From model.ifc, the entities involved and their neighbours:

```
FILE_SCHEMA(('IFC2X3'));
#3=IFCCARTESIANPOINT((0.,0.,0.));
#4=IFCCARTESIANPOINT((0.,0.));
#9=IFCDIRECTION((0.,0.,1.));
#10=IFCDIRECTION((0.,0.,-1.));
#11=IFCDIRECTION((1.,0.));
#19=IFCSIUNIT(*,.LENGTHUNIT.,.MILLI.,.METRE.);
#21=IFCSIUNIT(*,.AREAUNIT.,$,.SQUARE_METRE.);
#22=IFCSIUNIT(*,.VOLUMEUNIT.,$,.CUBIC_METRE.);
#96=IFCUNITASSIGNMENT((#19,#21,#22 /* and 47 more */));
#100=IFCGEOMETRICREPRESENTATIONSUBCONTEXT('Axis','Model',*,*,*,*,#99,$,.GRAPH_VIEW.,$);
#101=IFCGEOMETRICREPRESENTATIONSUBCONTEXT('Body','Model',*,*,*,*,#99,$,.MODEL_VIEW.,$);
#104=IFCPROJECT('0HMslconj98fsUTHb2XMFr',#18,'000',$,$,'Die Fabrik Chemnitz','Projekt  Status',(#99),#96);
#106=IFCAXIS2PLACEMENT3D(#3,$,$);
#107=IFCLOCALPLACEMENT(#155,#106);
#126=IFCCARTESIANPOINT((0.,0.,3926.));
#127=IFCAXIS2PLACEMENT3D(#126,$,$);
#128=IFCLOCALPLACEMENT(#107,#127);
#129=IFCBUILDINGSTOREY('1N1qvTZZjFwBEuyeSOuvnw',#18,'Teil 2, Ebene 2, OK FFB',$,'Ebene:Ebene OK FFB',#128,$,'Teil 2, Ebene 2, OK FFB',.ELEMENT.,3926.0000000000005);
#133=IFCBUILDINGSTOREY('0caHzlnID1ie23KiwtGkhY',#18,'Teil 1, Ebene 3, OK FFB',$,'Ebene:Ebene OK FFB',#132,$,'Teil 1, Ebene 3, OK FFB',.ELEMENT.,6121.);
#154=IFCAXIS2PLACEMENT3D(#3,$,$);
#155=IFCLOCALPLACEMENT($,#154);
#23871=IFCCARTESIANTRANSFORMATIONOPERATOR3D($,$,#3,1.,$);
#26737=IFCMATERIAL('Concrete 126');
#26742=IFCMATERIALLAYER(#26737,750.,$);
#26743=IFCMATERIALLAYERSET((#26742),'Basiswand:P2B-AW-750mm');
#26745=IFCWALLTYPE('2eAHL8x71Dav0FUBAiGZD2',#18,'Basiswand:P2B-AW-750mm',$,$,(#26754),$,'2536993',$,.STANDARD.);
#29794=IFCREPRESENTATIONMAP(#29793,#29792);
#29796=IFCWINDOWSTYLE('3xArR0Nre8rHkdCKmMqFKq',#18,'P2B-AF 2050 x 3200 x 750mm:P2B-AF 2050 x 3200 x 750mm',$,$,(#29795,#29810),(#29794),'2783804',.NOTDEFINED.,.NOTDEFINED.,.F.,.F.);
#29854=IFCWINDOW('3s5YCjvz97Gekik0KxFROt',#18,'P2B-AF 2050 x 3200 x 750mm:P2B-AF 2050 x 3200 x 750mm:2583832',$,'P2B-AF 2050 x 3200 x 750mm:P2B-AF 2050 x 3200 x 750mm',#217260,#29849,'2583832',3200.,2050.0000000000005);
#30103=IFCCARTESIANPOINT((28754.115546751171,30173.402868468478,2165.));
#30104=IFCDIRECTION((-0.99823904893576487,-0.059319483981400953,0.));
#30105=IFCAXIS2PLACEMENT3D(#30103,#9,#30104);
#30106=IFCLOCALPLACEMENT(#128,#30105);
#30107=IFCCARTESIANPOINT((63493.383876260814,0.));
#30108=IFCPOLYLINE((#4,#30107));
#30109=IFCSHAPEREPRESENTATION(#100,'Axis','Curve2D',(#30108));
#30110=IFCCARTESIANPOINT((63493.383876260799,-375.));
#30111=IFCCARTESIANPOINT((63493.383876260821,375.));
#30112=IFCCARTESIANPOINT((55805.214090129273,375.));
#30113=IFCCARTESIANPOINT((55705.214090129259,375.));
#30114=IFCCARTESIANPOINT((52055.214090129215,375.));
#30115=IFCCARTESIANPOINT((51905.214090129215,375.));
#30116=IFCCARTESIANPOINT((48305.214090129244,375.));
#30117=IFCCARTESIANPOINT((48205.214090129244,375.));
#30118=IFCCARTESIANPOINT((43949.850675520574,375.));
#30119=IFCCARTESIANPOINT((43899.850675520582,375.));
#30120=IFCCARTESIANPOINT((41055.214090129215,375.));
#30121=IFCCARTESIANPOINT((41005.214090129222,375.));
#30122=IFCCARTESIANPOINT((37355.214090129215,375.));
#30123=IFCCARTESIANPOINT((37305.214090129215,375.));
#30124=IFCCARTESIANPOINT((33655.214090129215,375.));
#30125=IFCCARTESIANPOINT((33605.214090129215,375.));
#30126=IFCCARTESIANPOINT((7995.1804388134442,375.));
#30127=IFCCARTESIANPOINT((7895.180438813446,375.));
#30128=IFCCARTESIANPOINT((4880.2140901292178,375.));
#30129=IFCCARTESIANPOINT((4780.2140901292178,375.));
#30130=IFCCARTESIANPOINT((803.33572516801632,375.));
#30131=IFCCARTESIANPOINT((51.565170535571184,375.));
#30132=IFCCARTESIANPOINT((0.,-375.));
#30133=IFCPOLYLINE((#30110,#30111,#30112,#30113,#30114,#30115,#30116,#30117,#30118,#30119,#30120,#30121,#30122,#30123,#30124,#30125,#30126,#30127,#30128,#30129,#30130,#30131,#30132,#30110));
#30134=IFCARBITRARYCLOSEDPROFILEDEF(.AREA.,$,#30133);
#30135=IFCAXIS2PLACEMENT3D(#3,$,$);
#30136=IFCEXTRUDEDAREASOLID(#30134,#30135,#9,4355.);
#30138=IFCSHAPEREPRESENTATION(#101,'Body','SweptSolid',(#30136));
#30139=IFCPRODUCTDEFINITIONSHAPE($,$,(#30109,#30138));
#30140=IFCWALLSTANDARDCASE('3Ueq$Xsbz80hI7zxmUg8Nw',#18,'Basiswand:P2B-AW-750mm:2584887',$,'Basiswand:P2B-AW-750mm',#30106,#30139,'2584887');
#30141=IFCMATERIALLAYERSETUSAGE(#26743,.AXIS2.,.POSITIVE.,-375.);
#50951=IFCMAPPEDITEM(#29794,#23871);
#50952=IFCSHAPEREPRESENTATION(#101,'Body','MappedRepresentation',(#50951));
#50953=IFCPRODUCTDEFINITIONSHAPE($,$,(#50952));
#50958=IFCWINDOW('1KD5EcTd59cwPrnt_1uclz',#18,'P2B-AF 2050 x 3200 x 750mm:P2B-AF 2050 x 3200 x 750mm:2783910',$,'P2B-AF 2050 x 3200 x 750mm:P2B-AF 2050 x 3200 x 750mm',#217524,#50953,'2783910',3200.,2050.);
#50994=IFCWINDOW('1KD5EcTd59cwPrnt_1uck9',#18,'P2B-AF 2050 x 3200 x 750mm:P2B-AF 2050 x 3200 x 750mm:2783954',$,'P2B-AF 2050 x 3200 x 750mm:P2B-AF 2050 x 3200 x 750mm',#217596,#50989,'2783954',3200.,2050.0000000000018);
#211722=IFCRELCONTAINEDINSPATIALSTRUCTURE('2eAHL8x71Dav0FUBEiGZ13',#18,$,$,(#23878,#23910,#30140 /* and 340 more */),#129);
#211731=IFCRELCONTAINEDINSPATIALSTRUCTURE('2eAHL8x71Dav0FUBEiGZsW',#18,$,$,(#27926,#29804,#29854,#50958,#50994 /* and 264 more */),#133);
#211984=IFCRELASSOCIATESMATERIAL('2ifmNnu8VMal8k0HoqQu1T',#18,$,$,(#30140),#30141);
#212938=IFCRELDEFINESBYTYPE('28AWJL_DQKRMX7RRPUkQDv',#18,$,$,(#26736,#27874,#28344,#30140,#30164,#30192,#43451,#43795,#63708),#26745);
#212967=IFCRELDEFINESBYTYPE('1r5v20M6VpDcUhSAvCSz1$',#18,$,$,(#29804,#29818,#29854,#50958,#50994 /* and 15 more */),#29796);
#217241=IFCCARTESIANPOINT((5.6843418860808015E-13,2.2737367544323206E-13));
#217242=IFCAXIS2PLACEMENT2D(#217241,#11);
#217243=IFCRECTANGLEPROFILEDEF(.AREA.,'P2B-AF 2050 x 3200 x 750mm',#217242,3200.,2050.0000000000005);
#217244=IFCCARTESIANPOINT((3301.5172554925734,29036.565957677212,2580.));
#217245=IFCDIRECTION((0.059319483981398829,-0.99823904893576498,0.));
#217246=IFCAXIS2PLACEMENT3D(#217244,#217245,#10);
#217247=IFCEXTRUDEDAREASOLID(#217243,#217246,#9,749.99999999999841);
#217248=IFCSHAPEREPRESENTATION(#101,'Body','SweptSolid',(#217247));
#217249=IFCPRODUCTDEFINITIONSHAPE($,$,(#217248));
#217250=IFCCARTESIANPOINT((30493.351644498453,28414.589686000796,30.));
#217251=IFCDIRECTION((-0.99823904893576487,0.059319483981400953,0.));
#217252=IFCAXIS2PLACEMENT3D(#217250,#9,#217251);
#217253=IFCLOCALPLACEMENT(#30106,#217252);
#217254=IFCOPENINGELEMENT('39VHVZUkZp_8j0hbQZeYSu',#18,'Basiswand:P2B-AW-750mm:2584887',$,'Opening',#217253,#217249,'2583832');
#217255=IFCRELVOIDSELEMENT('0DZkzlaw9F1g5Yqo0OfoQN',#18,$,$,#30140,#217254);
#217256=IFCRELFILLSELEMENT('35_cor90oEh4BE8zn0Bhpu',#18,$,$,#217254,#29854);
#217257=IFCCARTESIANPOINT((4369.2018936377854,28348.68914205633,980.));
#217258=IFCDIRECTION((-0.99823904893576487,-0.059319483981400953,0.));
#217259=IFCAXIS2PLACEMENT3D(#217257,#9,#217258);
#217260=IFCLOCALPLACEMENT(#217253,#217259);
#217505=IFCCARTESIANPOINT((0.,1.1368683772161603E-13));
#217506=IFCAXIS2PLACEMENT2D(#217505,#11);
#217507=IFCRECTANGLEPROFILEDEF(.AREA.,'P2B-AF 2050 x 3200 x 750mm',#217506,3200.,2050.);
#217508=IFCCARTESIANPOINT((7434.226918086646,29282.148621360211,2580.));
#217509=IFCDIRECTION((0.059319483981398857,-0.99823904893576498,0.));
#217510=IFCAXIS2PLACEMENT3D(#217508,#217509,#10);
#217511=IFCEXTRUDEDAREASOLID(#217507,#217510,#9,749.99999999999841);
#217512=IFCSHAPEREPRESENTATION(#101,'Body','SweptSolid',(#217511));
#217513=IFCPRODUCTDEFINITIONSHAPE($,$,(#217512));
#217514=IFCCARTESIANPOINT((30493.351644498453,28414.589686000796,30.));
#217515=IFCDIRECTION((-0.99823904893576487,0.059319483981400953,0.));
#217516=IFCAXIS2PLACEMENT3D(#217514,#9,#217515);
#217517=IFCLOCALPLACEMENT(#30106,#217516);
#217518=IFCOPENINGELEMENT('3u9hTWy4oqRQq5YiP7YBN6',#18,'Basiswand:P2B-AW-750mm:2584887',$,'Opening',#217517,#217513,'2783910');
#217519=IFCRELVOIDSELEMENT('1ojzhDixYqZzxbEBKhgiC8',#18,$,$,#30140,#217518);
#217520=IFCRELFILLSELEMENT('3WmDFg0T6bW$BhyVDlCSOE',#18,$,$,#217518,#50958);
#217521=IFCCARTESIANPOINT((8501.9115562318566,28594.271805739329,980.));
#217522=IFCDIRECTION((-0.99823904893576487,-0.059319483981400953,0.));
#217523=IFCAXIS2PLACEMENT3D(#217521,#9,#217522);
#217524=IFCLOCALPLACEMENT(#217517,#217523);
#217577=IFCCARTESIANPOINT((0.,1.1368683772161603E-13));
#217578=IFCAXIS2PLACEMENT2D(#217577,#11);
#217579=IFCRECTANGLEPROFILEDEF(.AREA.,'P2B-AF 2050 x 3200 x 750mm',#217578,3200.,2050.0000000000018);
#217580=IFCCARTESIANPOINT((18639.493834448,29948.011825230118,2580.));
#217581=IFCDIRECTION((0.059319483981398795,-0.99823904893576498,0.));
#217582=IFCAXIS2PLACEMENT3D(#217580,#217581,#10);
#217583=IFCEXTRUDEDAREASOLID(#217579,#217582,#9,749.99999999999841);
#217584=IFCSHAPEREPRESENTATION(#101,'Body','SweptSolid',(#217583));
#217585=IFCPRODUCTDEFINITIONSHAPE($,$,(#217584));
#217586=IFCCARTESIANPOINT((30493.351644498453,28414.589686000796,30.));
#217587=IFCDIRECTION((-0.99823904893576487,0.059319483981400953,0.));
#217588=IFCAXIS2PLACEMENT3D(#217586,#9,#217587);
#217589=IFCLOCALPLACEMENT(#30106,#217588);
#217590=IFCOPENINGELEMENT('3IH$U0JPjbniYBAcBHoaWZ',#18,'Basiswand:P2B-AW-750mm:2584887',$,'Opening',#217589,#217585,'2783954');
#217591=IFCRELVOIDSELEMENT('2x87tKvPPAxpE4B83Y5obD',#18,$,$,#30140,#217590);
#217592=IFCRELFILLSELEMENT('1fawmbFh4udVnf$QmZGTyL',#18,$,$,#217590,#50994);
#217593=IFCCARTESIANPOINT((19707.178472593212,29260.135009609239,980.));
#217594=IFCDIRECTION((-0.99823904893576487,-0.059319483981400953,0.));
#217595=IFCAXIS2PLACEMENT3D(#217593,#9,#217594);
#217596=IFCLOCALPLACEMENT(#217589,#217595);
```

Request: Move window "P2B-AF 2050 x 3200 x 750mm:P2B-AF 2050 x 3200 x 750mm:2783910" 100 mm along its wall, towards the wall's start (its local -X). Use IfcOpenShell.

```python
import ifcopenshell
import ifcopenshell.api.geometry
import ifcopenshell.util.placement
import ifcopenshell.util.unit

model = ifcopenshell.open("model.ifc")
unit_scale = ifcopenshell.util.unit.calculate_unit_scale(model)

window = model.by_guid("1KD5EcTd59cwPrnt_1uclz")
opening = window.FillsVoids[0].RelatingOpeningElement
wall = opening.VoidsElements[0].RelatingBuildingElement

wall_matrix = ifcopenshell.util.placement.get_local_placement(wall.ObjectPlacement)
shift = wall_matrix[:3, 0] * -0.1 / unit_scale
before = ifcopenshell.util.placement.get_local_placement(window.ObjectPlacement)[:3, 3].copy()

# The window is placed relative to its opening, so it follows when the opening moves.
matrix = ifcopenshell.util.placement.get_local_placement(opening.ObjectPlacement)
matrix[:3, 3] += shift
ifcopenshell.api.geometry.edit_object_placement(
    model, product=opening, matrix=matrix, is_si=False, should_transform_children=True
)

after = ifcopenshell.util.placement.get_local_placement(window.ObjectPlacement)[:3, 3]
print("window moved by", (after - before).round(3) + 0.0)

model.write("model_edited.ifc")
```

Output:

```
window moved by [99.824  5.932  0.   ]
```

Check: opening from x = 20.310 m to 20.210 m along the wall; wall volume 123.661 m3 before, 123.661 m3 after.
